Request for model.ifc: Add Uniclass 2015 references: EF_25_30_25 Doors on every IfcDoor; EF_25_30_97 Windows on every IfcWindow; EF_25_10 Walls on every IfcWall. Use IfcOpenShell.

First a look at what the model holds.

```python
import ifcopenshell

model = ifcopenshell.open("model.ifc")
print(model.schema)
print("classifications:", [c.Name for c in model.by_type("IfcClassification")])
for ifc_class in ("IfcDoor", "IfcRoof", "IfcStair", "IfcWall", "IfcWindow"):
    print(ifc_class, len(model.by_type(ifc_class)))
```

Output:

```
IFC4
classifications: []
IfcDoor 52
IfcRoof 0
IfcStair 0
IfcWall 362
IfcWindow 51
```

```python
import ifcopenshell
import ifcopenshell.api.classification

model = ifcopenshell.open("model.ifc")

system = ifcopenshell.api.classification.add_classification(model, classification="Uniclass 2015")

codes = {
    "IfcDoor": ("EF_25_30_25", "Doors"),
    "IfcWindow": ("EF_25_30_97", "Windows"),
    "IfcWall": ("EF_25_10", "Walls"),
}
for ifc_class, (code, name) in codes.items():
    products = model.by_type(ifc_class)
    ifcopenshell.api.classification.add_reference(
        model, products=products, classification=system, identification=code, name=name
    )
    print(code, len(products))

model.write("model_updated.ifc")
```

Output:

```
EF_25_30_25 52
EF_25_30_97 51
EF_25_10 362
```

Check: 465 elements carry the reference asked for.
